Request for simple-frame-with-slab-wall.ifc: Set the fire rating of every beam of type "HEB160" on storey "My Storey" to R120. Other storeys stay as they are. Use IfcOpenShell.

First a look at what the model holds.

```python
import ifcopenshell
import ifcopenshell.util.element

model = ifcopenshell.open("simple-frame-with-slab-wall.ifc")
print(model.schema)
storey = next(s for s in model.by_type("IfcBuildingStorey") if s.Name == "My Storey")
beams = [e for e in ifcopenshell.util.element.get_decomposition(storey) if e.is_a("IfcBeam")]
seen = {}
for e in beams:
    element_type = ifcopenshell.util.element.get_type(e)
    key = (element_type.Name if element_type != e and element_type else None, ifcopenshell.util.element.get_pset(e, "Pset_BeamCommon", "FireRating"))
    seen[key] = seen.get(key, 0) + 1
for (name, value), count in sorted(seen.items(), key=str):
    print(count, "x", name, "|", value)
```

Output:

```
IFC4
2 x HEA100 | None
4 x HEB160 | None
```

```python
import ifcopenshell
import ifcopenshell.api.pset
import ifcopenshell.util.element

model = ifcopenshell.open("simple-frame-with-slab-wall.ifc")

storey = next(s for s in model.by_type("IfcBuildingStorey") if s.Name == "My Storey")
beams = [e for e in ifcopenshell.util.element.get_decomposition(storey) if e.is_a("IfcBeam")]

count = 0
for e in beams:
    element_type = ifcopenshell.util.element.get_type(e)
    if element_type in (None, e) or element_type.Name != "HEB160":
        continue
    # add_pset returns the element's existing set when there is one.
    pset = ifcopenshell.api.pset.add_pset(model, product=e, name="Pset_BeamCommon")
    ifcopenshell.api.pset.edit_pset(model, pset=pset, properties={"FireRating": "R120"})
    count += 1

print(count, "beams updated")

model.write("simple-frame-with-slab-wall_rev.ifc")
```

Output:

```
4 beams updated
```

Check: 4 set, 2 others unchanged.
